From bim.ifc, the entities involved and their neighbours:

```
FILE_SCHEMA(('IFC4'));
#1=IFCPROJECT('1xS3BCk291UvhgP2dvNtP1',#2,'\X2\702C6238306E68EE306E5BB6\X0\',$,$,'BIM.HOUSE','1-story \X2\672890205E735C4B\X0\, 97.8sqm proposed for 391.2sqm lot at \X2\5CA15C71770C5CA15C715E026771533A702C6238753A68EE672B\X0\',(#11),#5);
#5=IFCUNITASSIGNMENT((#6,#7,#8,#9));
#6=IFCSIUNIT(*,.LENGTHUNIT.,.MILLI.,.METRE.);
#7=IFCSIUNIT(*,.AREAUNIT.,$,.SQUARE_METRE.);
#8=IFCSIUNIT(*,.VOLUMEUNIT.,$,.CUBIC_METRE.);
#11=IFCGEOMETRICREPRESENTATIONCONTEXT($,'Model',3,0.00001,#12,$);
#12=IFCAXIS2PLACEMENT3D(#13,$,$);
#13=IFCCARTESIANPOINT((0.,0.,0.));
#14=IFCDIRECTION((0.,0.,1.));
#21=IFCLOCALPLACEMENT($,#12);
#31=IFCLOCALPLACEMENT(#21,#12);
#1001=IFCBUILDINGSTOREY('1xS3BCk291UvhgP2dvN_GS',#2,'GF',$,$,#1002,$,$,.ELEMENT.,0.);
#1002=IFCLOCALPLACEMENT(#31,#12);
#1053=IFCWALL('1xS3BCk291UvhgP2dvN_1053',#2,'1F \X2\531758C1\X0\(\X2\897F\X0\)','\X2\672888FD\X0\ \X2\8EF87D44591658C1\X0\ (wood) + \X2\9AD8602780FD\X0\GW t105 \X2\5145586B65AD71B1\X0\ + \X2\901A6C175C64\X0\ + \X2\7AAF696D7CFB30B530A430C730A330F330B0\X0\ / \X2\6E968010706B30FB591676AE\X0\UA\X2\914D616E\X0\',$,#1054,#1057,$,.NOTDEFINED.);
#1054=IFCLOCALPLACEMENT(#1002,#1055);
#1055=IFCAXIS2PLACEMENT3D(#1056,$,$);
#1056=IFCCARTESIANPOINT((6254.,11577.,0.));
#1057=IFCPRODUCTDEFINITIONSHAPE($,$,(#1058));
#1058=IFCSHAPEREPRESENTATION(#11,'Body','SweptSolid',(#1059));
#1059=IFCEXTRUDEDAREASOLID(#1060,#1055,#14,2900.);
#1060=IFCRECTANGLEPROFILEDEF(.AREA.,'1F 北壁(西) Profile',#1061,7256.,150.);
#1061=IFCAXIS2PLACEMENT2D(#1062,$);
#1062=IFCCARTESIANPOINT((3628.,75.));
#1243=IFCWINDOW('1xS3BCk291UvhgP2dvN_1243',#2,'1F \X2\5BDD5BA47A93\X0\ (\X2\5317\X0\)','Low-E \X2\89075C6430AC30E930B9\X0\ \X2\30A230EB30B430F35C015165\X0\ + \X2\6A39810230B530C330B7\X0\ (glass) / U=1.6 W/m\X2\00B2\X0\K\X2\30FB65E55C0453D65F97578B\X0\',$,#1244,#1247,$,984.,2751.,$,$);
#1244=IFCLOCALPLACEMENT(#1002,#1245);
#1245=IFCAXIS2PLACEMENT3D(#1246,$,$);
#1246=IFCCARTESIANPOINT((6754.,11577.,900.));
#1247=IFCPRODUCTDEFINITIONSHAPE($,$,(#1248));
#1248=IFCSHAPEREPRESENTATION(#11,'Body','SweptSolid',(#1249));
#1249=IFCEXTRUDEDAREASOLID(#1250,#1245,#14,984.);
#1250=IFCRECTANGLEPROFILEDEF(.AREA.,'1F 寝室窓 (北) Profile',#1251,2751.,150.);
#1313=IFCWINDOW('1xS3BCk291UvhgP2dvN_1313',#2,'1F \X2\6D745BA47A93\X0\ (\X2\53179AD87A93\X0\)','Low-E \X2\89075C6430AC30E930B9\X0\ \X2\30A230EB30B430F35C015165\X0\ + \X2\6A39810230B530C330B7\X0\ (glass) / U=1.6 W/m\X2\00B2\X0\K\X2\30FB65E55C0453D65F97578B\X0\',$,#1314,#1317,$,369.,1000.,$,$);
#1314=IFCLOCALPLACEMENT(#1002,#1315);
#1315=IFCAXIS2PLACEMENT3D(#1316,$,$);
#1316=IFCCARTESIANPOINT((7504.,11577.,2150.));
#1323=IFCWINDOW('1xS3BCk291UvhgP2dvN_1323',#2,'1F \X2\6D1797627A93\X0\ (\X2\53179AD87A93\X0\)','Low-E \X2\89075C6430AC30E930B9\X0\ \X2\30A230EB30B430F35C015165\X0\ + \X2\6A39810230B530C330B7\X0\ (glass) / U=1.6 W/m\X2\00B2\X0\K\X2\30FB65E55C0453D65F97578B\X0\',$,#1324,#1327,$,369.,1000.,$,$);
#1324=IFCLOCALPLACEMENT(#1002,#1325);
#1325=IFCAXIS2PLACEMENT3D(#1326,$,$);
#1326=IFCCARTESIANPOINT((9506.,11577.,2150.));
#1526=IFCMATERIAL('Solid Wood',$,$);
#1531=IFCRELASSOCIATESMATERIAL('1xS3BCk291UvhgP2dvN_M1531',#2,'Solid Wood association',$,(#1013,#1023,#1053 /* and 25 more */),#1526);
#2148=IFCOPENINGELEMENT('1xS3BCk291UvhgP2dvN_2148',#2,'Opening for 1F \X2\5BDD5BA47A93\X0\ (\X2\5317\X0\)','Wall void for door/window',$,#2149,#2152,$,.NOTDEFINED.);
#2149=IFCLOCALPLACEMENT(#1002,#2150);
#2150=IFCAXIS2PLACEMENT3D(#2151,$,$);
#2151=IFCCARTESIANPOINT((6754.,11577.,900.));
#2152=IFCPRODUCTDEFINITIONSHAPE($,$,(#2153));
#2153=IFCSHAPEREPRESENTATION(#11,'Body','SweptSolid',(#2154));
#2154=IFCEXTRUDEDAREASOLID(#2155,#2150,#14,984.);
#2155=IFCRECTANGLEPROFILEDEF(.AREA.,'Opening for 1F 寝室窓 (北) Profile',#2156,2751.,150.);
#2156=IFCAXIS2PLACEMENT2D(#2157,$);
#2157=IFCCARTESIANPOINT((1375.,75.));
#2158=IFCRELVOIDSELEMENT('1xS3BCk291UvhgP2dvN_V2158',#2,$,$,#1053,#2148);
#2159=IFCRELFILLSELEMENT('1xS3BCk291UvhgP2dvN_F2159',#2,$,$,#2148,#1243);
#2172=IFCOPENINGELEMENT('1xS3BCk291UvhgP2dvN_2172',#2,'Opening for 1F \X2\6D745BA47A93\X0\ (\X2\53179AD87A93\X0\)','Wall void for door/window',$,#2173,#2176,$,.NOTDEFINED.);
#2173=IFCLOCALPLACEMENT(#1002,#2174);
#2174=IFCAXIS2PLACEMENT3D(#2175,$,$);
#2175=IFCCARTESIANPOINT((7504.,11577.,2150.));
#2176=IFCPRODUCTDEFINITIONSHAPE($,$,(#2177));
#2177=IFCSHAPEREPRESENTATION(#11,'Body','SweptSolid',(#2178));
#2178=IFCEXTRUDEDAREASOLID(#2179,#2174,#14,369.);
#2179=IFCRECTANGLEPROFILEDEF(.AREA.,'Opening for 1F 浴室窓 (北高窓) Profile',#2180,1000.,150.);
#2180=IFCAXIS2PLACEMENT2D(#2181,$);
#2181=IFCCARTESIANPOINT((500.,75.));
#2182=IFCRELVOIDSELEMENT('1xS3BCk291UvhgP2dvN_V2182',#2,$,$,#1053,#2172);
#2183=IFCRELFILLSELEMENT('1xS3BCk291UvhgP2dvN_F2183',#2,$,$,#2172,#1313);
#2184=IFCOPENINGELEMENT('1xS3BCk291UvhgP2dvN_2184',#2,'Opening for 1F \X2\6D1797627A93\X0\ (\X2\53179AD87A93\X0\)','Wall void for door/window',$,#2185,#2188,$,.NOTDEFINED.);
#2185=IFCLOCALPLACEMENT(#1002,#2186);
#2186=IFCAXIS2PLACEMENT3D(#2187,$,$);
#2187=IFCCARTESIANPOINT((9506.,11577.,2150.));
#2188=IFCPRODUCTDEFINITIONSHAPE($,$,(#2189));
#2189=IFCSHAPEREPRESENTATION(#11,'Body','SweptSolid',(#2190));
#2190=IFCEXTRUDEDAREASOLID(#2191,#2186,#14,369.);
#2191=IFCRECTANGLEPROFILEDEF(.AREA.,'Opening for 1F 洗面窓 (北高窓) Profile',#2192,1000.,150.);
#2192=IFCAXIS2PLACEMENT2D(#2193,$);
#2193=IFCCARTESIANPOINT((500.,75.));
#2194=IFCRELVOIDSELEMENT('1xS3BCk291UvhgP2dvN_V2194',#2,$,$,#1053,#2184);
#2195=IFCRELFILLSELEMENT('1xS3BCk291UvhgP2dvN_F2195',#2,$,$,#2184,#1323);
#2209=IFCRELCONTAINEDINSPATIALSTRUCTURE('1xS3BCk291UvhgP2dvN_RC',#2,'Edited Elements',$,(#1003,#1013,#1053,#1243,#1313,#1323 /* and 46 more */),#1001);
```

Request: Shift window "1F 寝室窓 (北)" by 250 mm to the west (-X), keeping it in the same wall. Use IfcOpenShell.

```python
import ifcopenshell
import ifcopenshell.api.geometry
import ifcopenshell.util.placement
import ifcopenshell.util.unit

model = ifcopenshell.open("bim.ifc")
unit_scale = ifcopenshell.util.unit.calculate_unit_scale(model)

window = model.by_id(1243)
opening = window.FillsVoids[0].RelatingOpeningElement
wall = opening.VoidsElements[0].RelatingBuildingElement

wall_matrix = ifcopenshell.util.placement.get_local_placement(wall.ObjectPlacement)
shift = wall_matrix[:3, 0] * -0.25 / unit_scale
before = ifcopenshell.util.placement.get_local_placement(window.ObjectPlacement)[:3, 3].copy()

# The window is not placed relative to its opening, so move both.
for product in (opening, window):
    matrix = ifcopenshell.util.placement.get_local_placement(product.ObjectPlacement)
    matrix[:3, 3] += shift
    ifcopenshell.api.geometry.edit_object_placement(model, product=product, matrix=matrix, is_si=False)

after = ifcopenshell.util.placement.get_local_placement(window.ObjectPlacement)[:3, 3]
print("window moved by", (after - before).round(3) + 0.0)

model.write("bim-out.ifc")
```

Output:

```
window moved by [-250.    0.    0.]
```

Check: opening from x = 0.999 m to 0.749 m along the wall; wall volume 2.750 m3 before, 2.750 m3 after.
